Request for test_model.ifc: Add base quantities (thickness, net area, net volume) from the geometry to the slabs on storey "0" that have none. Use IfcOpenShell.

First a look at what the model holds.

```python
import ifcopenshell
import ifcopenshell.util.element
import ifcopenshell.util.unit

model = ifcopenshell.open("test_model.ifc")
print(model.schema)
for unit_type in ("LENGTHUNIT", "AREAUNIT", "VOLUMEUNIT"):
    print(unit_type, ifcopenshell.util.unit.calculate_unit_scale(model, unit_type))
storey = next(s for s in model.by_type("IfcBuildingStorey") if s.Name == "0")
slabs = [e for e in ifcopenshell.util.element.get_decomposition(storey) if e.is_a("IfcSlab")]
for e in sorted(slabs, key=lambda e: e.id()):
    print(e.id(), e.is_a(), e.Name, list(ifcopenshell.util.element.get_psets(e, qtos_only=True)), sep=" | ")
```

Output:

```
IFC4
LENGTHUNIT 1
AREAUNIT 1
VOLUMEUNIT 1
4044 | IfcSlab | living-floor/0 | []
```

```python
import ifcopenshell
import ifcopenshell.api.pset
import ifcopenshell.geom
import ifcopenshell.util.element
import ifcopenshell.util.shape
import ifcopenshell.util.unit

model = ifcopenshell.open("test_model.ifc")
unit_scale = ifcopenshell.util.unit.calculate_unit_scale(model)
area_scale = ifcopenshell.util.unit.calculate_unit_scale(model, "AREAUNIT")
volume_scale = ifcopenshell.util.unit.calculate_unit_scale(model, "VOLUMEUNIT")
settings = ifcopenshell.geom.settings()

storey = next(s for s in model.by_type("IfcBuildingStorey") if s.Name == "0")
slabs = [e for e in ifcopenshell.util.element.get_decomposition(storey) if e.is_a("IfcSlab")]

for e in sorted(slabs, key=lambda e: e.id()):
    if ifcopenshell.util.element.get_psets(e, qtos_only=True, should_inherit=False):
        continue
    # Geometry comes back in metres, in the element's own axes.
    shape = ifcopenshell.geom.create_shape(settings, e)
    values = {
        "Width": ifcopenshell.util.shape.get_z(shape.geometry) / unit_scale,
        "NetArea": ifcopenshell.util.shape.get_footprint_area(shape.geometry) / area_scale,
        "NetVolume": ifcopenshell.util.shape.get_volume(shape.geometry) / volume_scale,
    }
    qto = ifcopenshell.api.pset.add_qto(model, product=e, name="Qto_SlabBaseQuantities")
    ifcopenshell.api.pset.edit_qto(model, qto=qto, properties=values)
    print(e.id(), {k: round(v, 3) for k, v in values.items()})

model.write("test_model_rev.ifc")
```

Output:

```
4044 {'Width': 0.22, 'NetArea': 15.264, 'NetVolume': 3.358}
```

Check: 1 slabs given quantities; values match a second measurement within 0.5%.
